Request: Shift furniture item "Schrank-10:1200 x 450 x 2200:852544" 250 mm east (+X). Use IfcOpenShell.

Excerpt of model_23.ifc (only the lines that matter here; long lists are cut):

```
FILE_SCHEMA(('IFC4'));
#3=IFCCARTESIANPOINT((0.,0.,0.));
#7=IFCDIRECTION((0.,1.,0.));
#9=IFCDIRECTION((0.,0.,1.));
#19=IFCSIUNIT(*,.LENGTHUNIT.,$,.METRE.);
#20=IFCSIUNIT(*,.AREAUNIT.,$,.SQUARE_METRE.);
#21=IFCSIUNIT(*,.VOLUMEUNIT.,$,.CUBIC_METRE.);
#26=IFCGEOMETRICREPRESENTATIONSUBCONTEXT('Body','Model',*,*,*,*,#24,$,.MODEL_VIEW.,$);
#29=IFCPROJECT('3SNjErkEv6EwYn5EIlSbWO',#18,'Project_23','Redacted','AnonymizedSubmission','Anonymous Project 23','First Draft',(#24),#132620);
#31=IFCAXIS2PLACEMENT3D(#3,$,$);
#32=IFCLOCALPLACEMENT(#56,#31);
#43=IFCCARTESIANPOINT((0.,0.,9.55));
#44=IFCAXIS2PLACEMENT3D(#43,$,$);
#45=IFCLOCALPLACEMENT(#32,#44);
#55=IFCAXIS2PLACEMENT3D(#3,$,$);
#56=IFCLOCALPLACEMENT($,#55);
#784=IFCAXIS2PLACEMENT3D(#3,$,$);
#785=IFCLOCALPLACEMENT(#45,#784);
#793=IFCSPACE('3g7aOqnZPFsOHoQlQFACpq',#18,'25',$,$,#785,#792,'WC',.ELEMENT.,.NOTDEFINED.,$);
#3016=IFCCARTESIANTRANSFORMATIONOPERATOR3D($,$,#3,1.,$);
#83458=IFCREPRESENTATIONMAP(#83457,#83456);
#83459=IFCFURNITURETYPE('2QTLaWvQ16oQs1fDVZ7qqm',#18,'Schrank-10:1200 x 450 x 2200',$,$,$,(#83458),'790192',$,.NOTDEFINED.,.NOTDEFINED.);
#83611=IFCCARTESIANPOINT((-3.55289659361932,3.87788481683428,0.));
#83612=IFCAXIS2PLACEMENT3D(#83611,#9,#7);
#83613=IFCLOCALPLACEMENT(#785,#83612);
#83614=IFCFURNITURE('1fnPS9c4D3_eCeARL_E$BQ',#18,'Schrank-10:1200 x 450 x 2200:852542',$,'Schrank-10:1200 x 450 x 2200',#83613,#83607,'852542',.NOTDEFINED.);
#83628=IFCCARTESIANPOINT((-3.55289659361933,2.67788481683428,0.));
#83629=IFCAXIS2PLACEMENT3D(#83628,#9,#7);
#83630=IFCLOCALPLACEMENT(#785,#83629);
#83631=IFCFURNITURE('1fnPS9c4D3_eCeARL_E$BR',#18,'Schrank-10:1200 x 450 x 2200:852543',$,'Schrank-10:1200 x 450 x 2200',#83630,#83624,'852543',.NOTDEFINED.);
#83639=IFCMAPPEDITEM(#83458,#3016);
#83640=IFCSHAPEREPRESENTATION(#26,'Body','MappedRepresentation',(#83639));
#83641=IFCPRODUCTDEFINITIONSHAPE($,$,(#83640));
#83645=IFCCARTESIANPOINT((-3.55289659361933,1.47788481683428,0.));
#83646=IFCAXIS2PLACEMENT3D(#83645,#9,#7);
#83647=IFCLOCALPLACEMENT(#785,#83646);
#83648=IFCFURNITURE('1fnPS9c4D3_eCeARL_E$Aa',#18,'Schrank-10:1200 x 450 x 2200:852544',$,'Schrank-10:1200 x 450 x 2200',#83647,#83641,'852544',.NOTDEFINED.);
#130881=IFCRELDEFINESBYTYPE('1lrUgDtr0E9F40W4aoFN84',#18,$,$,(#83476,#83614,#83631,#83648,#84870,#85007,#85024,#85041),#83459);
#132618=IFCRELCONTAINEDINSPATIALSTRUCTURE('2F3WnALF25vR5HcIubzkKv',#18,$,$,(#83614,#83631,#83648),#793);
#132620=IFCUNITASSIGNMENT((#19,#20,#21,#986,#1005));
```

```python
import ifcopenshell
import ifcopenshell.api.geometry
import ifcopenshell.util.placement
import ifcopenshell.util.unit

model = ifcopenshell.open("model_23.ifc")
unit_scale = ifcopenshell.util.unit.calculate_unit_scale(model)

item = model.by_id(83648)
matrix = ifcopenshell.util.placement.get_local_placement(item.ObjectPlacement)
matrix[0, 3] += 0.25 / unit_scale
ifcopenshell.api.geometry.edit_object_placement(model, product=item, matrix=matrix, is_si=False)

print(ifcopenshell.util.placement.get_local_placement(item.ObjectPlacement).round(3) + 0.0)

model.write("model_23-out.ifc")
```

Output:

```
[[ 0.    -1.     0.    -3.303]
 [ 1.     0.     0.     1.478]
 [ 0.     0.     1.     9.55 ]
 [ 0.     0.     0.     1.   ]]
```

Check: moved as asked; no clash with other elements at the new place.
